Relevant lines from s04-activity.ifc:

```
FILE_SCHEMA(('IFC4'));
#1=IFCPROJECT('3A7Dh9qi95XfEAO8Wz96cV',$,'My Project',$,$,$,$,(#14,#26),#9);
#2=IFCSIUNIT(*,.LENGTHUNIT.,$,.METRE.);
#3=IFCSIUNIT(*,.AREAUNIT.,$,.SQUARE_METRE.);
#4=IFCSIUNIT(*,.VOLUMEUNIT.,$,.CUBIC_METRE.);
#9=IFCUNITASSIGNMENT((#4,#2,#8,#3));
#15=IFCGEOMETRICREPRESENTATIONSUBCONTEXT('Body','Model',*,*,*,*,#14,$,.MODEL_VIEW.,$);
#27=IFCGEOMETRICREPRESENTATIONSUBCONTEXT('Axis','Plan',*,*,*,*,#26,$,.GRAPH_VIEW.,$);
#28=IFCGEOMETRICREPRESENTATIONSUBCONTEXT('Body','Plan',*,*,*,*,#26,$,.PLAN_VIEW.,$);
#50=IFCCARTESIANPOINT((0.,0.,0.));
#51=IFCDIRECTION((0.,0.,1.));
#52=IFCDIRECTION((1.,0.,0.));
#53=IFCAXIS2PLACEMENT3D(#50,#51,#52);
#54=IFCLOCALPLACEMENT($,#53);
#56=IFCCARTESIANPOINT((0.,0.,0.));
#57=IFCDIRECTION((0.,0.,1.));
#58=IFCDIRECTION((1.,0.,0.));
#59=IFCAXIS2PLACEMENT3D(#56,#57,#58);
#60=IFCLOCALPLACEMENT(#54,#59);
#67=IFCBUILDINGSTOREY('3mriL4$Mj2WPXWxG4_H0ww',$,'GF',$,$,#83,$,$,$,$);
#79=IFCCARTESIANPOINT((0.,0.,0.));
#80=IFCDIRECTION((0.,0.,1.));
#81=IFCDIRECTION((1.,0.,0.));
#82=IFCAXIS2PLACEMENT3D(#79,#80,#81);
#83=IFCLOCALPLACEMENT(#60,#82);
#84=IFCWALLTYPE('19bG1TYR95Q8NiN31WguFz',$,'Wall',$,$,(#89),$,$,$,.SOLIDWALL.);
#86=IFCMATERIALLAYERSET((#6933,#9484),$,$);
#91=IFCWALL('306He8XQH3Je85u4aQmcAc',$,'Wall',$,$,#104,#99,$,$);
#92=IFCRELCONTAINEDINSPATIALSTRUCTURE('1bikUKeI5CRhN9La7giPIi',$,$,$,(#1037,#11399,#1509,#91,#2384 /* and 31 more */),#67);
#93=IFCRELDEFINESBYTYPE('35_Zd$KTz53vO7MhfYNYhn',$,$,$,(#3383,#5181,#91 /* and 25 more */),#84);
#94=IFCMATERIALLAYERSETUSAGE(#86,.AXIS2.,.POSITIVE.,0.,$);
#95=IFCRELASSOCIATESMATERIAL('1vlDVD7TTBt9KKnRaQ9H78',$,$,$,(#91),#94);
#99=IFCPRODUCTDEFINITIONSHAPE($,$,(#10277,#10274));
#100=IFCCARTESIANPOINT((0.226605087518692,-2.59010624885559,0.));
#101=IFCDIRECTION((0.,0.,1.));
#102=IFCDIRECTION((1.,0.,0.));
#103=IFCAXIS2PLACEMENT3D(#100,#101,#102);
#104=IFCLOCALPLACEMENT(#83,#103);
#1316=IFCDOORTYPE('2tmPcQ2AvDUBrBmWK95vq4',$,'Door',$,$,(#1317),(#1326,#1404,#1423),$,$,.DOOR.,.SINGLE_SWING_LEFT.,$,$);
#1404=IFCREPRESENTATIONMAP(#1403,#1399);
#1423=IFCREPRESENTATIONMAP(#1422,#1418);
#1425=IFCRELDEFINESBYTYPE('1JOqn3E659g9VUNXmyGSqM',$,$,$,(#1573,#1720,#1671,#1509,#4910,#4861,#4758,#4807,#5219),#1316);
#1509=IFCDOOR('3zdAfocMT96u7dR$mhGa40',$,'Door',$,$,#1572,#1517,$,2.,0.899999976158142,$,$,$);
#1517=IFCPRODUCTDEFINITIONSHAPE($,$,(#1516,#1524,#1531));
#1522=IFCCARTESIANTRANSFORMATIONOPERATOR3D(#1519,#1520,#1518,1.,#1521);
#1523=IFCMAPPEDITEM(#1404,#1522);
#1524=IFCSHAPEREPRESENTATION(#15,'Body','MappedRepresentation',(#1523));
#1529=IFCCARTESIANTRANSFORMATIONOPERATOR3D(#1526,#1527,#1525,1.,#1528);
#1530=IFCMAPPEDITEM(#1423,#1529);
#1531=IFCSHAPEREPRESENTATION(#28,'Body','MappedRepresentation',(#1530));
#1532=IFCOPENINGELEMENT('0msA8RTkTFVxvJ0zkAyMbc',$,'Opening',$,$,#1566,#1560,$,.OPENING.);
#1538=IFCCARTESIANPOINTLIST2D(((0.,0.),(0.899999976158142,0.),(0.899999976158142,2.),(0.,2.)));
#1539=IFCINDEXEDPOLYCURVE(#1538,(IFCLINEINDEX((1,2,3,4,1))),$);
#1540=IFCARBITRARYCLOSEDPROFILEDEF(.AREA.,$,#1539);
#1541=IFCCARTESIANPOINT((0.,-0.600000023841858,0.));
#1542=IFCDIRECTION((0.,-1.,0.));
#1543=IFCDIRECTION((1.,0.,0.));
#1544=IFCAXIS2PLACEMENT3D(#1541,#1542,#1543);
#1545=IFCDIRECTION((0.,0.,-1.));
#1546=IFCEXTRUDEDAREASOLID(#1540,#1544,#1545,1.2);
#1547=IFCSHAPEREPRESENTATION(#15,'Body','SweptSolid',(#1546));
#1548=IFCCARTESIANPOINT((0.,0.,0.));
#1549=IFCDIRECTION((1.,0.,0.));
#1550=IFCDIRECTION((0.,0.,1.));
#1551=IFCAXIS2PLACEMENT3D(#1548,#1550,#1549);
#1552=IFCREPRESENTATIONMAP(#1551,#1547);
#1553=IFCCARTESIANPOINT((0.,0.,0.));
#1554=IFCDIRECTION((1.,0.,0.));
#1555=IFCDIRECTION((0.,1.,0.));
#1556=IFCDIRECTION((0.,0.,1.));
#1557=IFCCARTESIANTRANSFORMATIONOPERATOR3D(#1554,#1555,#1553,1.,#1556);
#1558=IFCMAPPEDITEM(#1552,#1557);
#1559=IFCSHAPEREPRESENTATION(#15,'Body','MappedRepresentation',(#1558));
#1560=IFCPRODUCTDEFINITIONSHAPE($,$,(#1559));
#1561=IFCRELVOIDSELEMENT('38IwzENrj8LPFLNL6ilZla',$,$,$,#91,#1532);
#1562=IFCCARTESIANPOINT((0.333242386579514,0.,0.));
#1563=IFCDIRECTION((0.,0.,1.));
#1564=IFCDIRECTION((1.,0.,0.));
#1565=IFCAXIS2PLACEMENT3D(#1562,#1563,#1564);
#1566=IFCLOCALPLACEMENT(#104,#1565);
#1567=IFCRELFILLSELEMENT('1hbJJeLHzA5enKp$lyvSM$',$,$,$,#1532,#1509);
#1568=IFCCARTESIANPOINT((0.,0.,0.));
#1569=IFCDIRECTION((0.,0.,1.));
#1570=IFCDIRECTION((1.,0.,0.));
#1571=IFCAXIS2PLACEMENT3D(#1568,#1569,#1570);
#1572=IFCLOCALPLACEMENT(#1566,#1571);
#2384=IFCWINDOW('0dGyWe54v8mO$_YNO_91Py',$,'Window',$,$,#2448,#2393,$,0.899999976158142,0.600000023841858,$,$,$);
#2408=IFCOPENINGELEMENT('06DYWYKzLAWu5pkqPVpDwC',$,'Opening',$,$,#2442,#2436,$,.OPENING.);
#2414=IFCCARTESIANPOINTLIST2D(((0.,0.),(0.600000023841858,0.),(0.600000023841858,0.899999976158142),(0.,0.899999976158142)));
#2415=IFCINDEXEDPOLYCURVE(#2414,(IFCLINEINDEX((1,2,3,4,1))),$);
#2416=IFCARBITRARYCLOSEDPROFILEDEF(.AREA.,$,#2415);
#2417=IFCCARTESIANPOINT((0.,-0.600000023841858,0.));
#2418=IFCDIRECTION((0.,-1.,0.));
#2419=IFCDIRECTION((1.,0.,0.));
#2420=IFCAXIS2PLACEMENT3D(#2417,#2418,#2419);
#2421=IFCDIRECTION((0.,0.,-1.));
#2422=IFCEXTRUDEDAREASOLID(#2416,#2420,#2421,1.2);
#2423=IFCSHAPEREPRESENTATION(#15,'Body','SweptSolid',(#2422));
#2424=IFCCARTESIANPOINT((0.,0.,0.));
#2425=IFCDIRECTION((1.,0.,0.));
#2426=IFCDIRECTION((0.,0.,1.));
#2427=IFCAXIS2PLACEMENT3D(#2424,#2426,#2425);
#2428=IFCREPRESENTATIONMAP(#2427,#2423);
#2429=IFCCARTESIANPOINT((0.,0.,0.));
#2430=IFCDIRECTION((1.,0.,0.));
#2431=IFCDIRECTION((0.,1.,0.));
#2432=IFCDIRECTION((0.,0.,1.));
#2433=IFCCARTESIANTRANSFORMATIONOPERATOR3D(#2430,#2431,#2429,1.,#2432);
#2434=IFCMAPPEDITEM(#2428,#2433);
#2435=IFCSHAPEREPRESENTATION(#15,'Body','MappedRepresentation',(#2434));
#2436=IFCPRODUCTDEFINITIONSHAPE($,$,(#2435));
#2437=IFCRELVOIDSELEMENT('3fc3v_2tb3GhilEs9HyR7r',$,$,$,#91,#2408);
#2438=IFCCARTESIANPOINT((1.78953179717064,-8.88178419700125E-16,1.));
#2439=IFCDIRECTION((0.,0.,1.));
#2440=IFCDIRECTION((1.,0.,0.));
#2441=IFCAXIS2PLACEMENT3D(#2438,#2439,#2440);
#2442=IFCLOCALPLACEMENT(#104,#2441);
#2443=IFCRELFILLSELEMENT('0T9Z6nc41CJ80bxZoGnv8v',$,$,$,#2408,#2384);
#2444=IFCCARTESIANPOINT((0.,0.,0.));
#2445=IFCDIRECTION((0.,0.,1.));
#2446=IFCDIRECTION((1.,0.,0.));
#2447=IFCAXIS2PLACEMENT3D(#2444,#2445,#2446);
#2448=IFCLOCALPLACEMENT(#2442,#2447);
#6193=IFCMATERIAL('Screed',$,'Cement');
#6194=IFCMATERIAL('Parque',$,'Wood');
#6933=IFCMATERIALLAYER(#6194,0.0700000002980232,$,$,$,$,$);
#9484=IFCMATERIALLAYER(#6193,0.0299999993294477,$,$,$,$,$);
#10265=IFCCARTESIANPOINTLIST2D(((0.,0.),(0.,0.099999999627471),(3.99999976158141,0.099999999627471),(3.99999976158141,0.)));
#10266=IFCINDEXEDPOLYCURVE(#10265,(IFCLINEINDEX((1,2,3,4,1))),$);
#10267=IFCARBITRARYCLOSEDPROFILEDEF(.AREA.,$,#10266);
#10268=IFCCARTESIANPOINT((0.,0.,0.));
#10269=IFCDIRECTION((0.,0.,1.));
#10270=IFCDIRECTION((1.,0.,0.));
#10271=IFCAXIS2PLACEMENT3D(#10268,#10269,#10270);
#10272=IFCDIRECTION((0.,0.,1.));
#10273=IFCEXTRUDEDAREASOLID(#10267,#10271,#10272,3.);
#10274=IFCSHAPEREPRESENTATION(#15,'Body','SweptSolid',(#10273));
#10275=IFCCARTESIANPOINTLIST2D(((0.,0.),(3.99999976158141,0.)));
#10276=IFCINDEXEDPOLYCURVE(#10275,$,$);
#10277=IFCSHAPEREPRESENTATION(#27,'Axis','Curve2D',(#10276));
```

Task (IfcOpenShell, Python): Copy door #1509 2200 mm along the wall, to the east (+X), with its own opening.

```python
import ifcopenshell
import ifcopenshell.api.feature
import ifcopenshell.api.geometry
import ifcopenshell.api.root
import ifcopenshell.geom
import ifcopenshell.util.element
import ifcopenshell.util.placement
import ifcopenshell.util.shape
import ifcopenshell.util.unit

model = ifcopenshell.open("s04-activity.ifc")
unit_scale = ifcopenshell.util.unit.calculate_unit_scale(model)
settings = ifcopenshell.geom.settings()


def volume(element):
    """Net volume in cubic metres, openings subtracted."""
    shape = ifcopenshell.geom.create_shape(settings, element)
    return ifcopenshell.util.shape.get_volume(shape.geometry)


door = model.by_guid("3zdAfocMT96u7dR$mhGa40")
opening = door.FillsVoids[0].RelatingOpeningElement
wall = opening.VoidsElements[0].RelatingBuildingElement
before = volume(wall)
shift = ifcopenshell.util.placement.get_local_placement(wall.ObjectPlacement)[:3, 0] * 2.2 / unit_scale

# copy_class copies the void relationship, type, container and properties, but no geometry.
new_opening = ifcopenshell.api.root.copy_class(model, product=opening)
new_opening.Representation = ifcopenshell.util.element.copy_deep(
    model, opening.Representation, exclude=["IfcGeometricRepresentationContext", "IfcRepresentationMap"]
)
new_door = ifcopenshell.api.root.copy_class(model, product=door)
new_door.Representation = ifcopenshell.util.element.copy_deep(
    model, door.Representation, exclude=["IfcGeometricRepresentationContext", "IfcRepresentationMap"]
)
ifcopenshell.api.feature.add_filling(model, opening=new_opening, element=new_door)

for old, new in ((opening, new_opening), (door, new_door)):
    matrix = ifcopenshell.util.placement.get_local_placement(old.ObjectPlacement)
    matrix[:3, 3] += shift
    ifcopenshell.api.geometry.edit_object_placement(model, product=new, matrix=matrix, is_si=False)

after = volume(wall)

print(f"wall volume {before:.3f} -> {after:.3f} m3")

model.write("s04-activity_rev.ifc")
```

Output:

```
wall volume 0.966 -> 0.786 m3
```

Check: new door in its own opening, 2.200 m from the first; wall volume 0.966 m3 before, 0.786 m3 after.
